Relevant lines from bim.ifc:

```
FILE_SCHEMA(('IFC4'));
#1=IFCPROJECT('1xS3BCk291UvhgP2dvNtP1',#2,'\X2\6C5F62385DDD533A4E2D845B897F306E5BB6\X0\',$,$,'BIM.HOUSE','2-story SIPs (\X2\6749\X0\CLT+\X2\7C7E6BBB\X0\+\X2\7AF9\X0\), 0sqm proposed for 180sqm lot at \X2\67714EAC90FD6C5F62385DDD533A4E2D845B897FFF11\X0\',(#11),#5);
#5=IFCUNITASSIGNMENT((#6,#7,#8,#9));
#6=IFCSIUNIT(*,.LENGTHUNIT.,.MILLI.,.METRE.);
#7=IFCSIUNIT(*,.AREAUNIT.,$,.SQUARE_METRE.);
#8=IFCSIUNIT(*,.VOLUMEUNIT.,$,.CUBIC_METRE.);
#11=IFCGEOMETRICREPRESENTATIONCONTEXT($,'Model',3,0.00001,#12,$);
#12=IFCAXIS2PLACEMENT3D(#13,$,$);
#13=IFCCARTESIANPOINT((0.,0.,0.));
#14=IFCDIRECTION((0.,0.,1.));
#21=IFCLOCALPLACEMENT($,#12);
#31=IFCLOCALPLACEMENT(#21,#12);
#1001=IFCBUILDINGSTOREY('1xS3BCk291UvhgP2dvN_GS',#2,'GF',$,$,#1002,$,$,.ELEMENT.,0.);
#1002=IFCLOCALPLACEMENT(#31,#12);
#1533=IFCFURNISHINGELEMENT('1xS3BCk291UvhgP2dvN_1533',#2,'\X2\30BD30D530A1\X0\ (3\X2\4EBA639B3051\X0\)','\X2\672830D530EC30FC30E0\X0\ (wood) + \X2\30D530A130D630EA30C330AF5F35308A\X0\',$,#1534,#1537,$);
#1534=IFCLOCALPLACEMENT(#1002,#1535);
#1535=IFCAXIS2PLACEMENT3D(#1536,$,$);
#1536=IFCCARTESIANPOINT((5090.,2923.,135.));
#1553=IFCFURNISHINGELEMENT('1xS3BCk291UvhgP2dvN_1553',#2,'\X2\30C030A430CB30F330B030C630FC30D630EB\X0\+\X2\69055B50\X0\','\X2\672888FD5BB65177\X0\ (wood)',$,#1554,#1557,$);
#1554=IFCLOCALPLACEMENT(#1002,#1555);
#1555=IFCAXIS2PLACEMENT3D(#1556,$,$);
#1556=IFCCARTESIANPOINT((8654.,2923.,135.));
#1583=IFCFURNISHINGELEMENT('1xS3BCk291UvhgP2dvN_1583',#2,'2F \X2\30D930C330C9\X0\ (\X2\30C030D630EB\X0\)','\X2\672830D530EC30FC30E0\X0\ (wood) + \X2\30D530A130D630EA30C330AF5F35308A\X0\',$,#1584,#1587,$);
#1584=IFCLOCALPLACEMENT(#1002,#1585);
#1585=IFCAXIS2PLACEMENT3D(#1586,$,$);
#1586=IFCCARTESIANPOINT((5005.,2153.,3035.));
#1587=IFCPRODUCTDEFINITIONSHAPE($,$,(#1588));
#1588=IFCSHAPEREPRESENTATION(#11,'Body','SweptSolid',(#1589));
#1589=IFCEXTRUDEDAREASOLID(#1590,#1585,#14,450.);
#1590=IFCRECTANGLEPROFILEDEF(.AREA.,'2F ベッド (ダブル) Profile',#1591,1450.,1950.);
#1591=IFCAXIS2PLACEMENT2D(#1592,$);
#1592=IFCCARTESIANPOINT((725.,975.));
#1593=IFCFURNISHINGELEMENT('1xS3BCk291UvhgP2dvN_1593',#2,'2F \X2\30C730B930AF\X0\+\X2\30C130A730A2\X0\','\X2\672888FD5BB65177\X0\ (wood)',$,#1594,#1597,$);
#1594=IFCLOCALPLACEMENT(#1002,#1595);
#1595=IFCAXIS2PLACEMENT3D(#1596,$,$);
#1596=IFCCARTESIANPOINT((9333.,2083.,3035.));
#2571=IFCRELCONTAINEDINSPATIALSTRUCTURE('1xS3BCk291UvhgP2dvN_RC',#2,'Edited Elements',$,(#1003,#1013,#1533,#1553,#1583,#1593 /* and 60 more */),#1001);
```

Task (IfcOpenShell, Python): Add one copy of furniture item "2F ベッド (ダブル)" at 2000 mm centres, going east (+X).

```python
import numpy as np
import ifcopenshell
import ifcopenshell.api.geometry
import ifcopenshell.api.root
import ifcopenshell.util.element
import ifcopenshell.util.placement
import ifcopenshell.util.unit

model = ifcopenshell.open("bim.ifc")
unit_scale = ifcopenshell.util.unit.calculate_unit_scale(model)


def reuse_history(source, copy):
    """copy_class also copies each property set's owner history, people and application; keep the originals."""
    for rel in copy.IsDefinedBy:
        if rel.is_a("IfcRelDefinesByProperties") and (history := rel.RelatingPropertyDefinition.OwnerHistory):
            rel.RelatingPropertyDefinition.OwnerHistory = source.OwnerHistory
            ifcopenshell.util.element.remove_deep2(model, history)


source = model.by_guid("1xS3BCk291UvhgP2dvN_1583")
base = ifcopenshell.util.placement.get_local_placement(source.ObjectPlacement)
step = np.array([1.0, 0.0, 0.0]) * 2 / unit_scale

for i in range(1, 2):
    copy = ifcopenshell.api.root.copy_class(model, product=source)
    copy.Representation = ifcopenshell.util.element.copy_deep(
        model, source.Representation, exclude=["IfcGeometricRepresentationContext", "IfcRepresentationMap"]
    )
    reuse_history(source, copy)
    matrix = base.copy()
    matrix[:3, 3] += i * step
    print("added at", matrix[:3, 3].round(3) + 0.0)
    ifcopenshell.api.geometry.edit_object_placement(model, product=copy, matrix=matrix, is_si=False)

model.write("bim_edited.ifc")
```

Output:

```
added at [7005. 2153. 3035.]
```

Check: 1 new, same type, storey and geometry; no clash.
